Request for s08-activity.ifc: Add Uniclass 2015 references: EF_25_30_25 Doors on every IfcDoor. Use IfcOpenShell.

First a look at what the model holds.

```python
import ifcopenshell

model = ifcopenshell.open("s08-activity.ifc")
print(model.schema)
print("classifications:", [c.Name for c in model.by_type("IfcClassification")])
for ifc_class in ("IfcDoor", "IfcRoof", "IfcStair", "IfcWall", "IfcWindow"):
    print(ifc_class, len(model.by_type(ifc_class)))
```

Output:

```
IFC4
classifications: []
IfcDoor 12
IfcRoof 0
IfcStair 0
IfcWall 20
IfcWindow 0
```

```python
import ifcopenshell
import ifcopenshell.api.classification

model = ifcopenshell.open("s08-activity.ifc")

system = ifcopenshell.api.classification.add_classification(model, classification="Uniclass 2015")

codes = {
    "IfcDoor": ("EF_25_30_25", "Doors"),
}
for ifc_class, (code, name) in codes.items():
    products = model.by_type(ifc_class)
    ifcopenshell.api.classification.add_reference(
        model, products=products, classification=system, identification=code, name=name
    )
    print(code, len(products))

model.write("s08-activity_edited.ifc")
```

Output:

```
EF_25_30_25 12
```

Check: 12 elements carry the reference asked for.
